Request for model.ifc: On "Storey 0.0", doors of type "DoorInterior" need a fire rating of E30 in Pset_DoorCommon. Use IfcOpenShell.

First a look at what the model holds.

```python
import ifcopenshell
import ifcopenshell.util.element

model = ifcopenshell.open("model.ifc")
print(model.schema)
storey = next(s for s in model.by_type("IfcBuildingStorey") if s.Name == "Storey 0.0")
doors = [e for e in ifcopenshell.util.element.get_decomposition(storey) if e.is_a("IfcDoor")]
seen = {}
for e in doors:
    element_type = ifcopenshell.util.element.get_type(e)
    key = (element_type.Name if element_type != e and element_type else None, ifcopenshell.util.element.get_pset(e, "Pset_DoorCommon", "FireRating"))
    seen[key] = seen.get(key, 0) + 1
for (name, value), count in sorted(seen.items(), key=str):
    print(count, "x", name, "|", value)
```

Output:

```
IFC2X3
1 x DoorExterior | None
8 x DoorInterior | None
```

```python
import ifcopenshell
import ifcopenshell.api.pset
import ifcopenshell.util.element

model = ifcopenshell.open("model.ifc")

storey = next(s for s in model.by_type("IfcBuildingStorey") if s.Name == "Storey 0.0")
doors = [e for e in ifcopenshell.util.element.get_decomposition(storey) if e.is_a("IfcDoor")]

count = 0
for e in doors:
    element_type = ifcopenshell.util.element.get_type(e)
    if element_type in (None, e) or element_type.Name != "DoorInterior":
        continue
    # add_pset returns the element's existing set when there is one.
    pset = ifcopenshell.api.pset.add_pset(model, product=e, name="Pset_DoorCommon")
    ifcopenshell.api.pset.edit_pset(model, pset=pset, properties={"FireRating": "E30"})
    count += 1

print(count, "doors updated")

model.write("model_edited.ifc")
```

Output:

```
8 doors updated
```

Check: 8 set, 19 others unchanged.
